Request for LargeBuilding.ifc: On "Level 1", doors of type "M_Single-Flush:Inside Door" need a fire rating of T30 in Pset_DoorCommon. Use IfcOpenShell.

First a look at what the model holds.

```python
import ifcopenshell
import ifcopenshell.util.element

model = ifcopenshell.open("LargeBuilding.ifc")
print(model.schema)
storey = next(s for s in model.by_type("IfcBuildingStorey") if s.Name == "Level 1")
doors = [e for e in ifcopenshell.util.element.get_decomposition(storey) if e.is_a("IfcDoor")]
seen = {}
for e in doors:
    element_type = ifcopenshell.util.element.get_type(e)
    key = (element_type.Name if element_type != e and element_type else None, ifcopenshell.util.element.get_pset(e, "Pset_DoorCommon", "FireRating"))
    seen[key] = seen.get(key, 0) + 1
for (name, value), count in sorted(seen.items(), key=str):
    print(count, "x", name, "|", value)
```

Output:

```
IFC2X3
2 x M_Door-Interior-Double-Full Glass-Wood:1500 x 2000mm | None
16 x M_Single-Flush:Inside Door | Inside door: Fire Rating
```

```python
import ifcopenshell
import ifcopenshell.api.pset
import ifcopenshell.util.element

model = ifcopenshell.open("LargeBuilding.ifc")

storey = next(s for s in model.by_type("IfcBuildingStorey") if s.Name == "Level 1")
doors = [e for e in ifcopenshell.util.element.get_decomposition(storey) if e.is_a("IfcDoor")]

count = 0
for e in doors:
    element_type = ifcopenshell.util.element.get_type(e)
    if element_type in (None, e) or element_type.Name != "M_Single-Flush:Inside Door":
        continue
    # add_pset returns the element's existing set when there is one.
    pset = ifcopenshell.api.pset.add_pset(model, product=e, name="Pset_DoorCommon")
    ifcopenshell.api.pset.edit_pset(model, pset=pset, properties={"FireRating": "T30"})
    count += 1

print(count, "doors updated")

model.write("LargeBuilding-out.ifc")
```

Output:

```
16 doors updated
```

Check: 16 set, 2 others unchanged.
